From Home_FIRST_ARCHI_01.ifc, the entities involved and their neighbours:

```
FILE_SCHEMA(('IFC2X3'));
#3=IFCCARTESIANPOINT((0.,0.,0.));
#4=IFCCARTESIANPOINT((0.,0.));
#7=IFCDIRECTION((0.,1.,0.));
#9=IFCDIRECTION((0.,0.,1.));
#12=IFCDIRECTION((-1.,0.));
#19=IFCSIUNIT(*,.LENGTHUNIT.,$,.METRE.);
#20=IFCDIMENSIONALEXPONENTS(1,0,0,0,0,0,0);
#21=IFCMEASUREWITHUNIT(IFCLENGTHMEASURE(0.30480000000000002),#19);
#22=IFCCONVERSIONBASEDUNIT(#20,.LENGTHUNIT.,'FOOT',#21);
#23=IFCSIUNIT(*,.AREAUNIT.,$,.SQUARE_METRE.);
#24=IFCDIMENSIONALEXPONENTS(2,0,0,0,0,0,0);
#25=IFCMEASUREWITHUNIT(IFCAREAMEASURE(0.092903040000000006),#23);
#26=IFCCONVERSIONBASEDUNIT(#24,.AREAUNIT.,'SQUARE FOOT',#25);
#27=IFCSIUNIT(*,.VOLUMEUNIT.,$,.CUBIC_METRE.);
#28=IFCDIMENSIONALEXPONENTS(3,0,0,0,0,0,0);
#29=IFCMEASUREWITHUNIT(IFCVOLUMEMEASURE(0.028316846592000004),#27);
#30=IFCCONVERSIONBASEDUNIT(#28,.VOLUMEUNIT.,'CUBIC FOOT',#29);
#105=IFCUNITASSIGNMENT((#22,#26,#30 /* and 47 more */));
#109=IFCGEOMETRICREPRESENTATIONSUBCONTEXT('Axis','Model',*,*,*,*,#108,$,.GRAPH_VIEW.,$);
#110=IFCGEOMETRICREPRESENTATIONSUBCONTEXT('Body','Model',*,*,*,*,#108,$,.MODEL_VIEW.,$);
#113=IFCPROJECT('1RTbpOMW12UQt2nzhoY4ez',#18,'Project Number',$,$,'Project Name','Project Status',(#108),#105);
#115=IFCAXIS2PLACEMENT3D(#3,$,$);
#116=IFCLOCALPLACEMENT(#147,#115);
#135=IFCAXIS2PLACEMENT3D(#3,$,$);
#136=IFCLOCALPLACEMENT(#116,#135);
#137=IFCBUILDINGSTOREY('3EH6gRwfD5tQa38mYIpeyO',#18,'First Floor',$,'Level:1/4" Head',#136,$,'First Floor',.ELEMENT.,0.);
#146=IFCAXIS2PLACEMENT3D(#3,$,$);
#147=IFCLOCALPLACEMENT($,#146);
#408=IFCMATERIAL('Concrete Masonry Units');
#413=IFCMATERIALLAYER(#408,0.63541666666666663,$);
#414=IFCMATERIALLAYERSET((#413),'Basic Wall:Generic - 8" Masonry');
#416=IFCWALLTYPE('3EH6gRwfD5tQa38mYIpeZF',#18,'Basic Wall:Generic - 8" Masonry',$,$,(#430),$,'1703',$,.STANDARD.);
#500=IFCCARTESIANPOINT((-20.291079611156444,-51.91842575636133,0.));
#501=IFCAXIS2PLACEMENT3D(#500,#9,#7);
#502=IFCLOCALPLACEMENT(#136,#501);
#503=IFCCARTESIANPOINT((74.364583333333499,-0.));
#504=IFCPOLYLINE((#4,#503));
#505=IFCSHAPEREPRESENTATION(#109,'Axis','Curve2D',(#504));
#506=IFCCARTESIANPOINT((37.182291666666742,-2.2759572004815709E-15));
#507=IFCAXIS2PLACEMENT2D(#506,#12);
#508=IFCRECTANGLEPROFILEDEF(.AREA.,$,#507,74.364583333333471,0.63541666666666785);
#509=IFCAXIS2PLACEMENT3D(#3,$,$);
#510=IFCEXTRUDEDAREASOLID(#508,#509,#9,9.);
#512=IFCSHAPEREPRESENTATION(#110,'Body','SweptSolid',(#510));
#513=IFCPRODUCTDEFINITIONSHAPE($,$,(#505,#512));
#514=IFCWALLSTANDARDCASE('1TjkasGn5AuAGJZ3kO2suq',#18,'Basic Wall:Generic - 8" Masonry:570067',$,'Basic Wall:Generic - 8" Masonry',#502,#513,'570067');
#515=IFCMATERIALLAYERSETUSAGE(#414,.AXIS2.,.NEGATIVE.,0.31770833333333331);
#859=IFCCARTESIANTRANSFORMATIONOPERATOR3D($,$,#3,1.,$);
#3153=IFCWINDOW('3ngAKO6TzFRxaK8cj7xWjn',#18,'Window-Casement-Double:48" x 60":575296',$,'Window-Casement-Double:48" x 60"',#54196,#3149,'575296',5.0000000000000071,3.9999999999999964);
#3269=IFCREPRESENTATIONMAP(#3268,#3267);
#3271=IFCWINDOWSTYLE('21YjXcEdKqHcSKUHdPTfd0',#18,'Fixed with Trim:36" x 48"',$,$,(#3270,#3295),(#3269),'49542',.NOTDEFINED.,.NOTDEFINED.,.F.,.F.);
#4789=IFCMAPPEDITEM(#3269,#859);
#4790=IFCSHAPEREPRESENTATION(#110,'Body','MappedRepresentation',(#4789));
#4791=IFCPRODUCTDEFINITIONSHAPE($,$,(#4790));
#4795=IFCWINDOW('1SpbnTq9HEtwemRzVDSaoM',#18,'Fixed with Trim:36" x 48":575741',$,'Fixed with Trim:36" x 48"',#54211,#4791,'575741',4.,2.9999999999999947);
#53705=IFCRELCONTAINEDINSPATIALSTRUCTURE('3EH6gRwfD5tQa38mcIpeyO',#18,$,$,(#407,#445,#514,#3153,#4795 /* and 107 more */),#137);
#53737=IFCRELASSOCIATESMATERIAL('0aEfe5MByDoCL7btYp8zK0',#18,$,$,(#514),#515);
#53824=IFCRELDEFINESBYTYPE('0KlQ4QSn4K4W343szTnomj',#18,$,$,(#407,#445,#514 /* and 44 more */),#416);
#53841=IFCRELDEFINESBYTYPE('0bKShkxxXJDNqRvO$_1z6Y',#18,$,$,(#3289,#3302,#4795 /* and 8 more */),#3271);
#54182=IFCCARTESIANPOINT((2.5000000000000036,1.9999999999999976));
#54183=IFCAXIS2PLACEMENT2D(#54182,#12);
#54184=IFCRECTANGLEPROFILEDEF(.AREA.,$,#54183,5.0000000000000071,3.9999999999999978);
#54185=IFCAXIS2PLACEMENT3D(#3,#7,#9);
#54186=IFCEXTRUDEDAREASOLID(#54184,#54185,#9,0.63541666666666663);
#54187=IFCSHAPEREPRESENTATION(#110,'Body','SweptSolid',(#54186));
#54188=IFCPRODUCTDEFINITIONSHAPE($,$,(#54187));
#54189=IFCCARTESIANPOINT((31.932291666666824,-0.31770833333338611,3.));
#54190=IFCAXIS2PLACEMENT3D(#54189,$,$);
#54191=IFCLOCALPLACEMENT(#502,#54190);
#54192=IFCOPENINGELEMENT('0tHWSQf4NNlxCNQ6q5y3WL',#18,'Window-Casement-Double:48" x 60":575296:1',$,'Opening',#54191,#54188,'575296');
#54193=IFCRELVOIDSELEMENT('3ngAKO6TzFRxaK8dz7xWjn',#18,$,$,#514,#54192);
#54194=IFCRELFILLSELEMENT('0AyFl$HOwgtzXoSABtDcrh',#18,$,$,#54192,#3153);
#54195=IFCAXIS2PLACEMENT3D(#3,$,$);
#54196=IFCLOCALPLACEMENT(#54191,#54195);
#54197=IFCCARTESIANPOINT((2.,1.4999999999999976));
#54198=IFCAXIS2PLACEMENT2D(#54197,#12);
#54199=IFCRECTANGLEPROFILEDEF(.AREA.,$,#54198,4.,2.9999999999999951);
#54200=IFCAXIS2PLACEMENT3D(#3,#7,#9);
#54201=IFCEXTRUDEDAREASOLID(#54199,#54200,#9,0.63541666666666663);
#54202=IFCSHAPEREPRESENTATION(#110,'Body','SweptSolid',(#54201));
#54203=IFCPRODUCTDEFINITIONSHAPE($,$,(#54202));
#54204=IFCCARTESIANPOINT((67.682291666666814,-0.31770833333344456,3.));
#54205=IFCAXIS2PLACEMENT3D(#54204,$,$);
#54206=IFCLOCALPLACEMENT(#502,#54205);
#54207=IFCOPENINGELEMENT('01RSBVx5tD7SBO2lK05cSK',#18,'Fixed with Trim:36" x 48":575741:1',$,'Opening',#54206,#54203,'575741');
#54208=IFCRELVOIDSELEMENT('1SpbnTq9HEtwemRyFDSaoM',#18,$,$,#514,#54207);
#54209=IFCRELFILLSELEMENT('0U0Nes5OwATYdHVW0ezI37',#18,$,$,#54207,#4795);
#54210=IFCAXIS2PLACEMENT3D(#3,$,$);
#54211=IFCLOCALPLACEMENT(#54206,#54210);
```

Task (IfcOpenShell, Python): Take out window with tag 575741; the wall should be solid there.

```python
import ifcopenshell
import ifcopenshell.api.feature
import ifcopenshell.api.root
import ifcopenshell.geom
import ifcopenshell.util.shape

model = ifcopenshell.open("Home_FIRST_ARCHI_01.ifc")
settings = ifcopenshell.geom.settings()


def volume(element):
    """Net volume in cubic metres, openings subtracted."""
    shape = ifcopenshell.geom.create_shape(settings, element)
    return ifcopenshell.util.shape.get_volume(shape.geometry)


window = model.by_guid("1SpbnTq9HEtwemRzVDSaoM")
opening = window.FillsVoids[0].RelatingOpeningElement
wall = opening.VoidsElements[0].RelatingBuildingElement
before = volume(wall)

ifcopenshell.api.root.remove_product(model, product=window)
ifcopenshell.api.feature.remove_feature(model, feature=opening)

after = volume(wall)

print(f"wall volume {before:.3f} -> {after:.3f} m3")

model.write("Home_FIRST_ARCHI_01_updated.ifc")
```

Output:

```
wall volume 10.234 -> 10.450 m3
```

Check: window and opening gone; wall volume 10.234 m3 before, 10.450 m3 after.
